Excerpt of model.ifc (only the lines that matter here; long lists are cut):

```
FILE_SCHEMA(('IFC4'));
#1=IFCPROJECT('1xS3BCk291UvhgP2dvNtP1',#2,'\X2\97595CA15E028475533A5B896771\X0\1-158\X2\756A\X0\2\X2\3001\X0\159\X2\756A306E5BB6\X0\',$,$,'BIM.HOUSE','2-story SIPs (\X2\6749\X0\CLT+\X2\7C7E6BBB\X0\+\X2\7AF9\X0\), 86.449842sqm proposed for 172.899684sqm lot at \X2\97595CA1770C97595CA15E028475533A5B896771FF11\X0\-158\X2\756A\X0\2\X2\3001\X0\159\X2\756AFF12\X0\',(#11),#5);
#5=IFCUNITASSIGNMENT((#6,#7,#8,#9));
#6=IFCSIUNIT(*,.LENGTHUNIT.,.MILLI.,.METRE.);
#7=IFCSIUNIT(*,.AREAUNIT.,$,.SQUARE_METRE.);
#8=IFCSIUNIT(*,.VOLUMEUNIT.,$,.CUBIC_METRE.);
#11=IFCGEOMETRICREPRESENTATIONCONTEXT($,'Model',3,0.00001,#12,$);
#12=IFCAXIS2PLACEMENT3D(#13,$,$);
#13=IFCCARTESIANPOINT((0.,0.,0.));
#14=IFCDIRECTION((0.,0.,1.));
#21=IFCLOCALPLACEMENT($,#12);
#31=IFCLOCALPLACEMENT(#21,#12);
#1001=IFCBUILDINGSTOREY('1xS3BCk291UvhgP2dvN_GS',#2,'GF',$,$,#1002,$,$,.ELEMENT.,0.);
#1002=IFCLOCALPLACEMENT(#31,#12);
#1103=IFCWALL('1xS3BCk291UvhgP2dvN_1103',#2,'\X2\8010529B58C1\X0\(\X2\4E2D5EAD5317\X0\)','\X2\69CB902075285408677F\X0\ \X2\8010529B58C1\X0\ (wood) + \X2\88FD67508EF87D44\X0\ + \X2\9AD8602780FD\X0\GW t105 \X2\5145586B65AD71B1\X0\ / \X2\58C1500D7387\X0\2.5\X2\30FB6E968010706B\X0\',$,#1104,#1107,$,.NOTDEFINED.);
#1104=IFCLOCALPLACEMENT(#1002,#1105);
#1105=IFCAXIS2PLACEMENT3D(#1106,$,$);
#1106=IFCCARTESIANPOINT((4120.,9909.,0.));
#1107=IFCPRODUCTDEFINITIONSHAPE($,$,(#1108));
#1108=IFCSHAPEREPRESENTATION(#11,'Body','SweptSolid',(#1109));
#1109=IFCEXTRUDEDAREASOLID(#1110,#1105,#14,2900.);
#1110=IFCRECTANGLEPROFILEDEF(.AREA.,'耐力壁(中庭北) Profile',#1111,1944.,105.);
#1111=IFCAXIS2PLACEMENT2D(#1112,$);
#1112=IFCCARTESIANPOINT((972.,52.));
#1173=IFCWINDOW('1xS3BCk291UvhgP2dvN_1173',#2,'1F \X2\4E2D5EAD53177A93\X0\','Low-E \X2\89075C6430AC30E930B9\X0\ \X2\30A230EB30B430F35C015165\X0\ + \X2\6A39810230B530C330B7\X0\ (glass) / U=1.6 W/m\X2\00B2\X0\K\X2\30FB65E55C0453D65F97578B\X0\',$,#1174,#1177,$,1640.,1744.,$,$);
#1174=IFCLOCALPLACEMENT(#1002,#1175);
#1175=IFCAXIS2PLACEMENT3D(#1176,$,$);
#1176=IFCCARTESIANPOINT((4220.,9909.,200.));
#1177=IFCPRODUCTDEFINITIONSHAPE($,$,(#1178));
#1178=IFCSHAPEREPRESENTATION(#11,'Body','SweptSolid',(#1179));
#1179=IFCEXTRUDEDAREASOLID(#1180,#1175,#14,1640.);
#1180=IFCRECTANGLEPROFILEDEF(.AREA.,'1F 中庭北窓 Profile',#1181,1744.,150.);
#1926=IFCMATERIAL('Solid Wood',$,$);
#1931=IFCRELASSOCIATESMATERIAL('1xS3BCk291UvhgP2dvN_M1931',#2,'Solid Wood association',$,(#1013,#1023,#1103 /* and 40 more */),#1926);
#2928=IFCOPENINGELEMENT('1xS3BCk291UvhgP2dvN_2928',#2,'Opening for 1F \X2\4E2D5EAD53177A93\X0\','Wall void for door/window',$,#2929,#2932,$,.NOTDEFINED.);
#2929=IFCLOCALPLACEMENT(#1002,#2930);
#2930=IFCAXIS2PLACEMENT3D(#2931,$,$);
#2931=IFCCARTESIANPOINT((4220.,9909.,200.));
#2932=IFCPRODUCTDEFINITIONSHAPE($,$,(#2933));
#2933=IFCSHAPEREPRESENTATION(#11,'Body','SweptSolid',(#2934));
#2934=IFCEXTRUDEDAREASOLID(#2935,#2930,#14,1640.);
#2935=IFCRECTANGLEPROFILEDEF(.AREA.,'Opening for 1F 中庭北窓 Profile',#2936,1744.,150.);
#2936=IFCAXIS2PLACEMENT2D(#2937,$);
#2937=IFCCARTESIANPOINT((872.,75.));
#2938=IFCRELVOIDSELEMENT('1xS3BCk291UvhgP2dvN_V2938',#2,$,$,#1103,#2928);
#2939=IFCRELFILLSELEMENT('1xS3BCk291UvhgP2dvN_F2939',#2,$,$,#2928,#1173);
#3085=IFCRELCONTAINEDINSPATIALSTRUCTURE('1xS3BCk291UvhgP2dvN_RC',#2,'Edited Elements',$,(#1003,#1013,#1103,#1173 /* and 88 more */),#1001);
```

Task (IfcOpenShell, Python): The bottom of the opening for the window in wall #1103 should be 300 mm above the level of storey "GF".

```python
import numpy as np
import ifcopenshell
import ifcopenshell.api.geometry
import ifcopenshell.geom
import ifcopenshell.util.element
import ifcopenshell.util.placement
import ifcopenshell.util.shape
import ifcopenshell.util.unit

model = ifcopenshell.open("model.ifc")
unit_scale = ifcopenshell.util.unit.calculate_unit_scale(model)

window = model.by_guid("1xS3BCk291UvhgP2dvN_1173")
opening = window.FillsVoids[0].RelatingOpeningElement
storey = ifcopenshell.util.element.get_container(window, ifc_class="IfcBuildingStorey")
level = ifcopenshell.util.placement.get_local_placement(storey.ObjectPlacement)[2, 3]

# The opening's origin need not be at the sill, so measure its lowest point.
shape = ifcopenshell.geom.create_shape(ifcopenshell.geom.settings(), opening)
bottom = ifcopenshell.util.shape.get_shape_bottom_elevation(shape, shape.geometry) / unit_scale
dz = level + 300.0 - bottom

shift = np.array([0.0, 0.0, dz])
# The window is not placed relative to its opening, so move both.
for product in (opening, window):
    matrix = ifcopenshell.util.placement.get_local_placement(product.ObjectPlacement)
    matrix[:3, 3] += shift
    ifcopenshell.api.geometry.edit_object_placement(model, product=product, matrix=matrix, is_si=False)

print(f"moved by {dz * unit_scale:+.3f} m")

model.write("model_updated.ifc")
```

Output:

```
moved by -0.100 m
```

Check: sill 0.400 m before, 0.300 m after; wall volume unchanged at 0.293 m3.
